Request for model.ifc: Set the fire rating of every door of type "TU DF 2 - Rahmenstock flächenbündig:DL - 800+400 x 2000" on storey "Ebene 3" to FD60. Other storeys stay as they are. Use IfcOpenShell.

First a look at what the model holds.

```python
import ifcopenshell
import ifcopenshell.util.element

model = ifcopenshell.open("model.ifc")
print(model.schema)
storey = next(s for s in model.by_type("IfcBuildingStorey") if s.Name == "Ebene 3")
doors = [e for e in ifcopenshell.util.element.get_decomposition(storey) if e.is_a("IfcDoor")]
seen = {}
for e in doors:
    element_type = ifcopenshell.util.element.get_type(e)
    key = (element_type.Name if element_type != e and element_type else None, ifcopenshell.util.element.get_pset(e, "Pset_DoorCommon", "FireRating"))
    seen[key] = seen.get(key, 0) + 1
for (name, value), count in sorted(seen.items(), key=str):
    print(count, "x", name, "|", value)
```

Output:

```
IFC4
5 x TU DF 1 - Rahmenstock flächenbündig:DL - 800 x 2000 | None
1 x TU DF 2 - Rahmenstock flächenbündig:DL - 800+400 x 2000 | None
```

```python
import ifcopenshell
import ifcopenshell.api.pset
import ifcopenshell.util.element

model = ifcopenshell.open("model.ifc")

storey = next(s for s in model.by_type("IfcBuildingStorey") if s.Name == "Ebene 3")
doors = [e for e in ifcopenshell.util.element.get_decomposition(storey) if e.is_a("IfcDoor")]

count = 0
for e in doors:
    element_type = ifcopenshell.util.element.get_type(e)
    if element_type in (None, e) or element_type.Name != "TU DF 2 - Rahmenstock flächenbündig:DL - 800+400 x 2000":
        continue
    # add_pset returns the element's existing set when there is one.
    pset = ifcopenshell.api.pset.add_pset(model, product=e, name="Pset_DoorCommon")
    ifcopenshell.api.pset.edit_pset(model, pset=pset, properties={"FireRating": "FD60"})
    count += 1

print(count, "doors updated")

model.write("model_v2.ifc")
```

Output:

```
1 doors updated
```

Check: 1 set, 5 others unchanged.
